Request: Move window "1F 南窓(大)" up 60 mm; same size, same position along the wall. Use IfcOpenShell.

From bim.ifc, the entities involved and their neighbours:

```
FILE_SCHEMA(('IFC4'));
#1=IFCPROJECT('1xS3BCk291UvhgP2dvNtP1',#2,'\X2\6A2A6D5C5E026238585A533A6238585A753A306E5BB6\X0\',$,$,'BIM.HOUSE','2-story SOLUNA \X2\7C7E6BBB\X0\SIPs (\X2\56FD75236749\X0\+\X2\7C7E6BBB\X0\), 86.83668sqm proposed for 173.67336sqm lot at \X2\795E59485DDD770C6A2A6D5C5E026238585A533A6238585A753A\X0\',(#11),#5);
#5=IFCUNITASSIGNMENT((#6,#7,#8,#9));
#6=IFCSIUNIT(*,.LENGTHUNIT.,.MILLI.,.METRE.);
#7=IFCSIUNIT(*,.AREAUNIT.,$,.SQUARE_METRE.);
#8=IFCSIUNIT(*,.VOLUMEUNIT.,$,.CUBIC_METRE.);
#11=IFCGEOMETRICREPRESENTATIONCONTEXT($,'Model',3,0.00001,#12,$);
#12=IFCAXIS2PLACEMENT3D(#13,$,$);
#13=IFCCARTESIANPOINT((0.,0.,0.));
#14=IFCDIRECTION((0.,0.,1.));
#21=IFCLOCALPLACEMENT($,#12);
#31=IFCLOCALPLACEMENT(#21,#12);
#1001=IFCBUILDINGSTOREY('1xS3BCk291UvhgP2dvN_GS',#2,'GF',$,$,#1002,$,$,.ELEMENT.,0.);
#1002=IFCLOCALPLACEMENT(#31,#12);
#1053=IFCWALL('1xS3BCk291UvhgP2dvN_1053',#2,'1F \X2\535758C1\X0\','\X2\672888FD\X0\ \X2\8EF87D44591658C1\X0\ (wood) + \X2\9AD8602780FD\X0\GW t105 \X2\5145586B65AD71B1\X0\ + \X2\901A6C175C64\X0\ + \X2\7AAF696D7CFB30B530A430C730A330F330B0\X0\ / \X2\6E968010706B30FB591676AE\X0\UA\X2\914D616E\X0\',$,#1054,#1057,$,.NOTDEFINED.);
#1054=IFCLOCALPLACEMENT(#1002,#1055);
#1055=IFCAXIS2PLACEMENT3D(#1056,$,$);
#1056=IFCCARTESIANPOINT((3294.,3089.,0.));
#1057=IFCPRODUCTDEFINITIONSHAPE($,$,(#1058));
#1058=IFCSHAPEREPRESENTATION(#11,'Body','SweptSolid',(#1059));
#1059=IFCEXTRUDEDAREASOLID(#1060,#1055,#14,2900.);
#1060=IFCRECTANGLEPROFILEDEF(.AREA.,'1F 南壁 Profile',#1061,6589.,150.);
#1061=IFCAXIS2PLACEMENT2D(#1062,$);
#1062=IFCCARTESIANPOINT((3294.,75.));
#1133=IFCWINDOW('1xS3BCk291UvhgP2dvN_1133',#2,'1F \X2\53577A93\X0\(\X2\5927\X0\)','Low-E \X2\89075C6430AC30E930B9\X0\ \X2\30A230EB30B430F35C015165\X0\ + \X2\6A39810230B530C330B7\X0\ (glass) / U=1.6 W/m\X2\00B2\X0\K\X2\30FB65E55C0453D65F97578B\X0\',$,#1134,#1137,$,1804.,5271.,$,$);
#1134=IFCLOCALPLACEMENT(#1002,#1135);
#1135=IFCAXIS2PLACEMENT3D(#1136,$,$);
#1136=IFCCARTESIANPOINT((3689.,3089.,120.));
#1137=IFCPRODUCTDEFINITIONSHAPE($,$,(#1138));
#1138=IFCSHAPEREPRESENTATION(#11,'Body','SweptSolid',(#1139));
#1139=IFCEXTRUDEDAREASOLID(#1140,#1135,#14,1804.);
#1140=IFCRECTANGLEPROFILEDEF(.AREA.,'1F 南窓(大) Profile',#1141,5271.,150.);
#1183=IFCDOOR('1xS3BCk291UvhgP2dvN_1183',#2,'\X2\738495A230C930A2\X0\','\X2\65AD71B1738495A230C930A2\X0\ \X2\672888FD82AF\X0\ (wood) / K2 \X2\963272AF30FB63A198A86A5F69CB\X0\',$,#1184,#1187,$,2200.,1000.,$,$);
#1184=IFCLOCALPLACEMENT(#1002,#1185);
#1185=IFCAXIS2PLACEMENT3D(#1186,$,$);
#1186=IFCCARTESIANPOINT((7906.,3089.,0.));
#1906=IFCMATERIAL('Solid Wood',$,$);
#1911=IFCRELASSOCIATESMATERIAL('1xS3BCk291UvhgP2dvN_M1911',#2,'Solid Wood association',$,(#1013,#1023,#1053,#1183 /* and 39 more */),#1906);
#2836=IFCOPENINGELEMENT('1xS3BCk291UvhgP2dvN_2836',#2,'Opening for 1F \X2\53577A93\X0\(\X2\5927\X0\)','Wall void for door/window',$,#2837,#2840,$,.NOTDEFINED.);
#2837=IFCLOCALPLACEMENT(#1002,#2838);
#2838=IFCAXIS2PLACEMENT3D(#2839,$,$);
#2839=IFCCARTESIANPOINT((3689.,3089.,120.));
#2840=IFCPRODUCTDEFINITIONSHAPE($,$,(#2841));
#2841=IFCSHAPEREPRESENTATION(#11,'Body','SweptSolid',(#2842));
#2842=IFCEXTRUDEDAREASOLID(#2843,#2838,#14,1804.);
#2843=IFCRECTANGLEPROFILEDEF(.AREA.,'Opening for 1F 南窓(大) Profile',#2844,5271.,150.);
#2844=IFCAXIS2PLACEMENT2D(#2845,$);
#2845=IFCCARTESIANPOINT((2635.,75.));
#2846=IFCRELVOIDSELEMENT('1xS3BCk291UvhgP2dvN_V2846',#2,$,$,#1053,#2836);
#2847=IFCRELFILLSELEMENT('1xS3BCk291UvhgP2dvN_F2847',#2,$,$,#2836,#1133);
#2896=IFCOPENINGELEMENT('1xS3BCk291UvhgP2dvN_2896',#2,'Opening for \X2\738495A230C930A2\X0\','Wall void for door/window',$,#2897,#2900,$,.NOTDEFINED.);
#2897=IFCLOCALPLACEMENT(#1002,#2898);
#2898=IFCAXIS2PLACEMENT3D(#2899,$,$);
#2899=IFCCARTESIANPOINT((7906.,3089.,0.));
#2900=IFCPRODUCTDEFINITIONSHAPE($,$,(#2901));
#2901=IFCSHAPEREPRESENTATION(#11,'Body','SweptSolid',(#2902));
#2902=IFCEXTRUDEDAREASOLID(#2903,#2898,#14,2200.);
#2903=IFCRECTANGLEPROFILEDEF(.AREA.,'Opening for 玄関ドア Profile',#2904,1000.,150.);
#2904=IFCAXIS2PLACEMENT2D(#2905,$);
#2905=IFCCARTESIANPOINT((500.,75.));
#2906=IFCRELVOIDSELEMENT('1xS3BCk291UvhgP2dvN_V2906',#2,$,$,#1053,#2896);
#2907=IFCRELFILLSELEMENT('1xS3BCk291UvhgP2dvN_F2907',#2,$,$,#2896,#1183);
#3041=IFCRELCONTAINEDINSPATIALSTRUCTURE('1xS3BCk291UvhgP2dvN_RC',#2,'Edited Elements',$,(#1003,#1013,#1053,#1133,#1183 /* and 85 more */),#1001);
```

```python
import numpy as np
import ifcopenshell
import ifcopenshell.api.geometry
import ifcopenshell.util.placement
import ifcopenshell.util.unit

model = ifcopenshell.open("bim.ifc")
unit_scale = ifcopenshell.util.unit.calculate_unit_scale(model)

window = model.by_id(1133)
opening = window.FillsVoids[0].RelatingOpeningElement
dz = 0.06 / unit_scale

shift = np.array([0.0, 0.0, dz])
# The window is not placed relative to its opening, so move both.
for product in (opening, window):
    matrix = ifcopenshell.util.placement.get_local_placement(product.ObjectPlacement)
    matrix[:3, 3] += shift
    ifcopenshell.api.geometry.edit_object_placement(model, product=product, matrix=matrix, is_si=False)

print(f"moved by {dz * unit_scale:+.3f} m")

model.write("bim-out.ifc")
```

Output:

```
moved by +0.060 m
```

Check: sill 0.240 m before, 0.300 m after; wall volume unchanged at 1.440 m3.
